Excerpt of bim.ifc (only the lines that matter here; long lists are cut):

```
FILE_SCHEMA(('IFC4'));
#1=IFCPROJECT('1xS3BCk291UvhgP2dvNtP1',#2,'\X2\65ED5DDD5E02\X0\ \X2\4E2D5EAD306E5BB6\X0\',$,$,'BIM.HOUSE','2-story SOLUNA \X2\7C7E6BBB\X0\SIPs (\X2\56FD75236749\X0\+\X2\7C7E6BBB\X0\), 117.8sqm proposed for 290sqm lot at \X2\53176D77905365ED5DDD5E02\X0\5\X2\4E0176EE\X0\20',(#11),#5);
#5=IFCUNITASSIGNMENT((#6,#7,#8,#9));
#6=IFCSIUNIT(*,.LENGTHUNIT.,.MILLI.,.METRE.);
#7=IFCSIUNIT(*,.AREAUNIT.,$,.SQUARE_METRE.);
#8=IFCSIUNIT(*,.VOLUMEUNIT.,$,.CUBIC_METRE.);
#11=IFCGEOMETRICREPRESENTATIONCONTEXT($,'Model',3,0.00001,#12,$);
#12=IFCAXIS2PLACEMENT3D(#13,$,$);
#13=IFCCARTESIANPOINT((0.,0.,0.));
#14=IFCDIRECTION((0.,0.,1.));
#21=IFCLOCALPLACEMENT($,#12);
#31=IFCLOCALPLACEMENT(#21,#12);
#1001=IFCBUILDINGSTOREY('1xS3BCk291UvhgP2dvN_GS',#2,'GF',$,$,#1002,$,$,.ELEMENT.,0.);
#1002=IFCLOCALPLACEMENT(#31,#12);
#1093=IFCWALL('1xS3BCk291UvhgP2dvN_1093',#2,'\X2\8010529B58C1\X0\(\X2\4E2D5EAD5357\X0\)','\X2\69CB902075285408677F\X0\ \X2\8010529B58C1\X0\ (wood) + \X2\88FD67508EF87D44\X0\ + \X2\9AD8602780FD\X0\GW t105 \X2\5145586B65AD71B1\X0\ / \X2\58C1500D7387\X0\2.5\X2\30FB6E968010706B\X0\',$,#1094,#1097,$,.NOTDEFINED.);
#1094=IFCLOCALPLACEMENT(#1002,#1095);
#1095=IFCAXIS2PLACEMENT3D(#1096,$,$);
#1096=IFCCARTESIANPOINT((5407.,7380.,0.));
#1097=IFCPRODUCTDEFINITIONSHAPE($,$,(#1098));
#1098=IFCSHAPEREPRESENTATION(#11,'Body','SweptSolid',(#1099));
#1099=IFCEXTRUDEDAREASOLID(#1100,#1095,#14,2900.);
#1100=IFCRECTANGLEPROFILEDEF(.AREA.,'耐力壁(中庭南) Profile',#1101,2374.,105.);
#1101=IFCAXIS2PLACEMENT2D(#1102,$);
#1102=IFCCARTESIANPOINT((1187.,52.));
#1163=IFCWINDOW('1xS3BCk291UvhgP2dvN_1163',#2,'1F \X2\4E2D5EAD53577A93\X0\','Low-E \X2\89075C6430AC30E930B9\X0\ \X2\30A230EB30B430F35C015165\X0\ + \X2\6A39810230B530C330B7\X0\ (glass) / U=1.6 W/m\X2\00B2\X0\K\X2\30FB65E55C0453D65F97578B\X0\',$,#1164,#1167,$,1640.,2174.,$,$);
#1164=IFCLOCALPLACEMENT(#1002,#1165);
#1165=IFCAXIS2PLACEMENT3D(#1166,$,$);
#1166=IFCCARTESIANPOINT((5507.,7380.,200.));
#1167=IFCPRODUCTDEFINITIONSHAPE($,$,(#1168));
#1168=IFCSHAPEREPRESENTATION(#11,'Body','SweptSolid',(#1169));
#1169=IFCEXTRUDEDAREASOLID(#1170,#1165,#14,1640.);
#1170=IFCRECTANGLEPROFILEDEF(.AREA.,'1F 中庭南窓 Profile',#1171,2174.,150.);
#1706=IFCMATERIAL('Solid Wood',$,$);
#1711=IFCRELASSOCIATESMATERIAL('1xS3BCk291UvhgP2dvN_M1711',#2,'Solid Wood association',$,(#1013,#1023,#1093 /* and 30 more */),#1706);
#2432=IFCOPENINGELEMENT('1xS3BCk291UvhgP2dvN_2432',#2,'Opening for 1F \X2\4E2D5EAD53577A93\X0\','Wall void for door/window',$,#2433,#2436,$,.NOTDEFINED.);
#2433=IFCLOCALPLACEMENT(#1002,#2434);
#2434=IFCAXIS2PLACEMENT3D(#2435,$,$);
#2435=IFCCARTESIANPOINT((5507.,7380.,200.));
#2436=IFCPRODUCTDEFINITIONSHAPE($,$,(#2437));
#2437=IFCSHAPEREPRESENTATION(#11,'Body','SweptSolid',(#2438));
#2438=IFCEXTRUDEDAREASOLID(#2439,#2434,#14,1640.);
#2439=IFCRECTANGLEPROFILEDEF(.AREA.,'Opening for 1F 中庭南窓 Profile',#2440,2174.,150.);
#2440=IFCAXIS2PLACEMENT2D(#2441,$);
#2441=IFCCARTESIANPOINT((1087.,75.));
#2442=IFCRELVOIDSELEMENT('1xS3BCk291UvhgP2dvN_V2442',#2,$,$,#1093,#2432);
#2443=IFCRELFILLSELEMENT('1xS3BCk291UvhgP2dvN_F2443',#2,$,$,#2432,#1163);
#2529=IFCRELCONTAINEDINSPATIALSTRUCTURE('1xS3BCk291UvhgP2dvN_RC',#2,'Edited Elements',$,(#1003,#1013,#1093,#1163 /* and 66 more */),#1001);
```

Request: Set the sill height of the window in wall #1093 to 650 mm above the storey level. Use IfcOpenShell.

```python
import numpy as np
import ifcopenshell
import ifcopenshell.api.geometry
import ifcopenshell.geom
import ifcopenshell.util.element
import ifcopenshell.util.placement
import ifcopenshell.util.shape
import ifcopenshell.util.unit

model = ifcopenshell.open("bim.ifc")
unit_scale = ifcopenshell.util.unit.calculate_unit_scale(model)

window = model.by_guid("1xS3BCk291UvhgP2dvN_1163")
opening = window.FillsVoids[0].RelatingOpeningElement
storey = ifcopenshell.util.element.get_container(window, ifc_class="IfcBuildingStorey")
level = ifcopenshell.util.placement.get_local_placement(storey.ObjectPlacement)[2, 3]

# The opening's origin need not be at the sill, so measure its lowest point.
shape = ifcopenshell.geom.create_shape(ifcopenshell.geom.settings(), opening)
bottom = ifcopenshell.util.shape.get_shape_bottom_elevation(shape, shape.geometry) / unit_scale
dz = level + 0.65 / unit_scale - bottom

shift = np.array([0.0, 0.0, dz])
# The window is not placed relative to its opening, so move both.
for product in (opening, window):
    matrix = ifcopenshell.util.placement.get_local_placement(product.ObjectPlacement)
    matrix[:3, 3] += shift
    ifcopenshell.api.geometry.edit_object_placement(model, product=product, matrix=matrix, is_si=False)

print(f"moved by {dz * unit_scale:+.3f} m")

model.write("bim_updated.ifc")
```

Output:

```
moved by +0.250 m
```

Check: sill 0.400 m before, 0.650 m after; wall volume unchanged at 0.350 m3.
